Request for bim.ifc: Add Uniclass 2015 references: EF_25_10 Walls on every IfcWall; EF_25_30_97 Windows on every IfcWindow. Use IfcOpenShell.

First a look at what the model holds.

```python
import ifcopenshell

model = ifcopenshell.open("bim.ifc")
print(model.schema)
print("classifications:", [c.Name for c in model.by_type("IfcClassification")])
for ifc_class in ("IfcDoor", "IfcRoof", "IfcStair", "IfcWall", "IfcWindow"):
    print(ifc_class, len(model.by_type(ifc_class)))
```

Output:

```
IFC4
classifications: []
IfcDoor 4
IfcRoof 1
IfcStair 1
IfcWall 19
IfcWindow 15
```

```python
import ifcopenshell
import ifcopenshell.api.classification

model = ifcopenshell.open("bim.ifc")

system = ifcopenshell.api.classification.add_classification(model, classification="Uniclass 2015")

codes = {
    "IfcWall": ("EF_25_10", "Walls"),
    "IfcWindow": ("EF_25_30_97", "Windows"),
}
for ifc_class, (code, name) in codes.items():
    products = model.by_type(ifc_class)
    ifcopenshell.api.classification.add_reference(
        model, products=products, classification=system, identification=code, name=name
    )
    print(code, len(products))

model.write("bim-out.ifc")
```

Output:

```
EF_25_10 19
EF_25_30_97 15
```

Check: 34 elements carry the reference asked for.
